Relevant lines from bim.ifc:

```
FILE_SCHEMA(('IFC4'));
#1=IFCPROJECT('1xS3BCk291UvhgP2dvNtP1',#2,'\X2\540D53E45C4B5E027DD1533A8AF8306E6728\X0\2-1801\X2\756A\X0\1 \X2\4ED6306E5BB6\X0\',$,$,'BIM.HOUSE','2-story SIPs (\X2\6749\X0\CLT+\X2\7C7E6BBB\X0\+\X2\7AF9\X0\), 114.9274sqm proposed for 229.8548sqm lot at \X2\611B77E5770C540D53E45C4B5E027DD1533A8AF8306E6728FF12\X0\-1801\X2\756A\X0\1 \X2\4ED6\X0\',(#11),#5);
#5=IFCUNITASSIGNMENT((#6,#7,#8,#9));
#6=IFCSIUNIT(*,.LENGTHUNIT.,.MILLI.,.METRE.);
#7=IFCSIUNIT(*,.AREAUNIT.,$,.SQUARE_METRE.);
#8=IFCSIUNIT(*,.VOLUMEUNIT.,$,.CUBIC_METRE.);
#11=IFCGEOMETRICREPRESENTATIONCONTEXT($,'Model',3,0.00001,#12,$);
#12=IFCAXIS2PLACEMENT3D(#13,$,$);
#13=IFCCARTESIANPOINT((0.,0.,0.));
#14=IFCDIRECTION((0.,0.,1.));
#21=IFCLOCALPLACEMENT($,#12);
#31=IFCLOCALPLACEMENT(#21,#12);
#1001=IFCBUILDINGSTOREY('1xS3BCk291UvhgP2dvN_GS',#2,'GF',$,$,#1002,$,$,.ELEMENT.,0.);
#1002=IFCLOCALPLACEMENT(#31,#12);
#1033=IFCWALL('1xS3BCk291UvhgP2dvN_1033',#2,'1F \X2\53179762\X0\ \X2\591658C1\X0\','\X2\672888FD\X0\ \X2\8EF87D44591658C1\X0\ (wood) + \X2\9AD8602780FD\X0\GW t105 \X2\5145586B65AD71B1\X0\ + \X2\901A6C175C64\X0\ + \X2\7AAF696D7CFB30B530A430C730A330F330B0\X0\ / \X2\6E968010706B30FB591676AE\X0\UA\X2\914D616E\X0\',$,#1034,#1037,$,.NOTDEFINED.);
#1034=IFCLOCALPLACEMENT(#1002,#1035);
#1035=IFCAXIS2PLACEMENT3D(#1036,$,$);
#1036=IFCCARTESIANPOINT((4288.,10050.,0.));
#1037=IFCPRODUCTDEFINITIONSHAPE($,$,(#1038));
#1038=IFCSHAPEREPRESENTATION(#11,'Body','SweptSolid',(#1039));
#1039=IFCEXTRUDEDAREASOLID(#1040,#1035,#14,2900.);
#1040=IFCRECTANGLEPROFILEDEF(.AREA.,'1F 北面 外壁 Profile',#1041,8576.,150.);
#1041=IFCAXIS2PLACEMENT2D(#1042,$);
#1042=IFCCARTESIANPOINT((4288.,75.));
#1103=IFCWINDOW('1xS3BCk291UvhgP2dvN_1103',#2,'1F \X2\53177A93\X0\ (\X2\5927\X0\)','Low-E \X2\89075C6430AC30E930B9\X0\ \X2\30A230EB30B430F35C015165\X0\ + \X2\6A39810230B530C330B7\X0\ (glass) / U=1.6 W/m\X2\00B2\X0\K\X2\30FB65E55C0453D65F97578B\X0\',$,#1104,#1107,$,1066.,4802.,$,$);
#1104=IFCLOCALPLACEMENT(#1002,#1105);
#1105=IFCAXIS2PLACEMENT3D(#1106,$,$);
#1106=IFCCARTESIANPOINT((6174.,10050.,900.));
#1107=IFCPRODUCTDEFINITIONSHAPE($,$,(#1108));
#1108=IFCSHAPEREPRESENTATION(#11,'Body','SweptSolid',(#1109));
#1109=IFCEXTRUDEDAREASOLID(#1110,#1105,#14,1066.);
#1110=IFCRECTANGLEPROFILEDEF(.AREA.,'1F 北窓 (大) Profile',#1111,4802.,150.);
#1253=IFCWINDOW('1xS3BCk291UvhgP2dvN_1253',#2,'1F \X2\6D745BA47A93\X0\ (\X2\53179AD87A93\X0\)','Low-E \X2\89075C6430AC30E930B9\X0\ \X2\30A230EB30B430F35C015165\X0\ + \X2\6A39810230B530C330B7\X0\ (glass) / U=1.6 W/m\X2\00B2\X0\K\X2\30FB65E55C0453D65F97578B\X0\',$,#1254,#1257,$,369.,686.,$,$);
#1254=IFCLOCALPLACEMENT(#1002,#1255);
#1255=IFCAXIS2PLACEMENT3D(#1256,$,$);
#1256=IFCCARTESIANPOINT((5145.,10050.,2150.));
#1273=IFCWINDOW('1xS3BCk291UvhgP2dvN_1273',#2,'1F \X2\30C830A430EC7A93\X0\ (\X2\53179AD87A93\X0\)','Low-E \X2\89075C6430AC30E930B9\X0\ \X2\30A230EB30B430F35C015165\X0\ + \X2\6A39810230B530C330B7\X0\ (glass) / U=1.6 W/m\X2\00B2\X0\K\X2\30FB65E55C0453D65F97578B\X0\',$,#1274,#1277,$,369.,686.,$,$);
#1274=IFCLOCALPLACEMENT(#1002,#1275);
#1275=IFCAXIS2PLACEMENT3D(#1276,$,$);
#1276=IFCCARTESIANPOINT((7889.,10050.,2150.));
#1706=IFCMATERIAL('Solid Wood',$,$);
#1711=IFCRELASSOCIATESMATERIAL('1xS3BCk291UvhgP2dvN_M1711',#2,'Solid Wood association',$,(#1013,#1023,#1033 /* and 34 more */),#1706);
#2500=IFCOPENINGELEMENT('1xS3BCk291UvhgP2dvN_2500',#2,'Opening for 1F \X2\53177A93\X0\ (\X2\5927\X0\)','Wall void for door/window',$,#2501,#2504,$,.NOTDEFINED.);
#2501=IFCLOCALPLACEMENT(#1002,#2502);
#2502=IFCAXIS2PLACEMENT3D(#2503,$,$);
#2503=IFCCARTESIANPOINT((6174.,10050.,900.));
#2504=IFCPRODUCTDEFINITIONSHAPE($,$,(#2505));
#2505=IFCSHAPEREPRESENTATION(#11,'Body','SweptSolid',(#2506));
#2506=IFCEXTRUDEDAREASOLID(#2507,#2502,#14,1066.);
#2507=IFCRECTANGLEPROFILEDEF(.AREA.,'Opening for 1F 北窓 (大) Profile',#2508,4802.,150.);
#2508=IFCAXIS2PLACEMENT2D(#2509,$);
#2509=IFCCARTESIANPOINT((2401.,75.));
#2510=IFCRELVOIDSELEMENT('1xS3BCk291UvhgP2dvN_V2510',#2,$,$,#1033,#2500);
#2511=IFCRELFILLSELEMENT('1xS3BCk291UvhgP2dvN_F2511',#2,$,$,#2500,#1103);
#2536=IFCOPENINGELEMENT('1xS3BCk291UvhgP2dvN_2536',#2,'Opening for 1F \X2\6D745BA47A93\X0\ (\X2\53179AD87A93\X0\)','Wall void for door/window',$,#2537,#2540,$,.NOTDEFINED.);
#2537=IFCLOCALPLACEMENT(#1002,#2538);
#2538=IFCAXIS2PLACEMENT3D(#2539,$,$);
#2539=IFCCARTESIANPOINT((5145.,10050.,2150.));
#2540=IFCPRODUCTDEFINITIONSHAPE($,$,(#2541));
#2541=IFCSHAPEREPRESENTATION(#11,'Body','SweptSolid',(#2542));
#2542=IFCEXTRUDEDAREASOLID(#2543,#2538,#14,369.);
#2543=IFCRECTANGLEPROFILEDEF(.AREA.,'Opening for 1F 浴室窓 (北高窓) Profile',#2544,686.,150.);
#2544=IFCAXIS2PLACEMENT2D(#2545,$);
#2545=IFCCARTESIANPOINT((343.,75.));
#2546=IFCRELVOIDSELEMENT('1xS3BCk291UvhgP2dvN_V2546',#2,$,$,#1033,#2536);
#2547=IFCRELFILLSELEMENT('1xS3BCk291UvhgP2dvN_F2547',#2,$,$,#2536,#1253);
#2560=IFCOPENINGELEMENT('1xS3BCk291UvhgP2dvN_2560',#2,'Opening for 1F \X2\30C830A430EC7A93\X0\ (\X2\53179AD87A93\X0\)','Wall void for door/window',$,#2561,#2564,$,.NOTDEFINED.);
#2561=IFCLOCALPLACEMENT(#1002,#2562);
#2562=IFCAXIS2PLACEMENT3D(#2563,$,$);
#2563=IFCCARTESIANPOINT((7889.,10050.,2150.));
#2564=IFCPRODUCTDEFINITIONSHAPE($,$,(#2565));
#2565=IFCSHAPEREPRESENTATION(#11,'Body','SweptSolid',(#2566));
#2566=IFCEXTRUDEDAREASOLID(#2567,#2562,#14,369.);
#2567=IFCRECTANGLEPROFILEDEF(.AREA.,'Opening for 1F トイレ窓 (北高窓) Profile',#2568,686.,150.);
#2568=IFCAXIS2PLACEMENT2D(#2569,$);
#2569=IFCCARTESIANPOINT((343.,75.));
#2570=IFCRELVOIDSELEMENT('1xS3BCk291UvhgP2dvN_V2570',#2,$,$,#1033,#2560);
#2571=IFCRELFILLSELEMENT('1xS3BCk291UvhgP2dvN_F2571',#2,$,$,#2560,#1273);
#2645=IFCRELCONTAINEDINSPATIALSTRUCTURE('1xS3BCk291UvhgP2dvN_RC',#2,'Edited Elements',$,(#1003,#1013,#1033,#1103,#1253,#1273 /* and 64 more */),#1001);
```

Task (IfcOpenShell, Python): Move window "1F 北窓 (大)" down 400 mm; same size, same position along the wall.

```python
import numpy as np
import ifcopenshell
import ifcopenshell.api.geometry
import ifcopenshell.util.placement
import ifcopenshell.util.unit

model = ifcopenshell.open("bim.ifc")
unit_scale = ifcopenshell.util.unit.calculate_unit_scale(model)

window = model.by_guid("1xS3BCk291UvhgP2dvN_1103")
opening = window.FillsVoids[0].RelatingOpeningElement
dz = -0.4 / unit_scale

shift = np.array([0.0, 0.0, dz])
# The window is not placed relative to its opening, so move both.
for product in (opening, window):
    matrix = ifcopenshell.util.placement.get_local_placement(product.ObjectPlacement)
    matrix[:3, 3] += shift
    ifcopenshell.api.geometry.edit_object_placement(model, product=product, matrix=matrix, is_si=False)

print(f"moved by {dz * unit_scale:+.3f} m")

model.write("bim_updated.ifc")
```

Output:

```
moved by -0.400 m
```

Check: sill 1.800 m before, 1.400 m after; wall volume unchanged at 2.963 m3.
